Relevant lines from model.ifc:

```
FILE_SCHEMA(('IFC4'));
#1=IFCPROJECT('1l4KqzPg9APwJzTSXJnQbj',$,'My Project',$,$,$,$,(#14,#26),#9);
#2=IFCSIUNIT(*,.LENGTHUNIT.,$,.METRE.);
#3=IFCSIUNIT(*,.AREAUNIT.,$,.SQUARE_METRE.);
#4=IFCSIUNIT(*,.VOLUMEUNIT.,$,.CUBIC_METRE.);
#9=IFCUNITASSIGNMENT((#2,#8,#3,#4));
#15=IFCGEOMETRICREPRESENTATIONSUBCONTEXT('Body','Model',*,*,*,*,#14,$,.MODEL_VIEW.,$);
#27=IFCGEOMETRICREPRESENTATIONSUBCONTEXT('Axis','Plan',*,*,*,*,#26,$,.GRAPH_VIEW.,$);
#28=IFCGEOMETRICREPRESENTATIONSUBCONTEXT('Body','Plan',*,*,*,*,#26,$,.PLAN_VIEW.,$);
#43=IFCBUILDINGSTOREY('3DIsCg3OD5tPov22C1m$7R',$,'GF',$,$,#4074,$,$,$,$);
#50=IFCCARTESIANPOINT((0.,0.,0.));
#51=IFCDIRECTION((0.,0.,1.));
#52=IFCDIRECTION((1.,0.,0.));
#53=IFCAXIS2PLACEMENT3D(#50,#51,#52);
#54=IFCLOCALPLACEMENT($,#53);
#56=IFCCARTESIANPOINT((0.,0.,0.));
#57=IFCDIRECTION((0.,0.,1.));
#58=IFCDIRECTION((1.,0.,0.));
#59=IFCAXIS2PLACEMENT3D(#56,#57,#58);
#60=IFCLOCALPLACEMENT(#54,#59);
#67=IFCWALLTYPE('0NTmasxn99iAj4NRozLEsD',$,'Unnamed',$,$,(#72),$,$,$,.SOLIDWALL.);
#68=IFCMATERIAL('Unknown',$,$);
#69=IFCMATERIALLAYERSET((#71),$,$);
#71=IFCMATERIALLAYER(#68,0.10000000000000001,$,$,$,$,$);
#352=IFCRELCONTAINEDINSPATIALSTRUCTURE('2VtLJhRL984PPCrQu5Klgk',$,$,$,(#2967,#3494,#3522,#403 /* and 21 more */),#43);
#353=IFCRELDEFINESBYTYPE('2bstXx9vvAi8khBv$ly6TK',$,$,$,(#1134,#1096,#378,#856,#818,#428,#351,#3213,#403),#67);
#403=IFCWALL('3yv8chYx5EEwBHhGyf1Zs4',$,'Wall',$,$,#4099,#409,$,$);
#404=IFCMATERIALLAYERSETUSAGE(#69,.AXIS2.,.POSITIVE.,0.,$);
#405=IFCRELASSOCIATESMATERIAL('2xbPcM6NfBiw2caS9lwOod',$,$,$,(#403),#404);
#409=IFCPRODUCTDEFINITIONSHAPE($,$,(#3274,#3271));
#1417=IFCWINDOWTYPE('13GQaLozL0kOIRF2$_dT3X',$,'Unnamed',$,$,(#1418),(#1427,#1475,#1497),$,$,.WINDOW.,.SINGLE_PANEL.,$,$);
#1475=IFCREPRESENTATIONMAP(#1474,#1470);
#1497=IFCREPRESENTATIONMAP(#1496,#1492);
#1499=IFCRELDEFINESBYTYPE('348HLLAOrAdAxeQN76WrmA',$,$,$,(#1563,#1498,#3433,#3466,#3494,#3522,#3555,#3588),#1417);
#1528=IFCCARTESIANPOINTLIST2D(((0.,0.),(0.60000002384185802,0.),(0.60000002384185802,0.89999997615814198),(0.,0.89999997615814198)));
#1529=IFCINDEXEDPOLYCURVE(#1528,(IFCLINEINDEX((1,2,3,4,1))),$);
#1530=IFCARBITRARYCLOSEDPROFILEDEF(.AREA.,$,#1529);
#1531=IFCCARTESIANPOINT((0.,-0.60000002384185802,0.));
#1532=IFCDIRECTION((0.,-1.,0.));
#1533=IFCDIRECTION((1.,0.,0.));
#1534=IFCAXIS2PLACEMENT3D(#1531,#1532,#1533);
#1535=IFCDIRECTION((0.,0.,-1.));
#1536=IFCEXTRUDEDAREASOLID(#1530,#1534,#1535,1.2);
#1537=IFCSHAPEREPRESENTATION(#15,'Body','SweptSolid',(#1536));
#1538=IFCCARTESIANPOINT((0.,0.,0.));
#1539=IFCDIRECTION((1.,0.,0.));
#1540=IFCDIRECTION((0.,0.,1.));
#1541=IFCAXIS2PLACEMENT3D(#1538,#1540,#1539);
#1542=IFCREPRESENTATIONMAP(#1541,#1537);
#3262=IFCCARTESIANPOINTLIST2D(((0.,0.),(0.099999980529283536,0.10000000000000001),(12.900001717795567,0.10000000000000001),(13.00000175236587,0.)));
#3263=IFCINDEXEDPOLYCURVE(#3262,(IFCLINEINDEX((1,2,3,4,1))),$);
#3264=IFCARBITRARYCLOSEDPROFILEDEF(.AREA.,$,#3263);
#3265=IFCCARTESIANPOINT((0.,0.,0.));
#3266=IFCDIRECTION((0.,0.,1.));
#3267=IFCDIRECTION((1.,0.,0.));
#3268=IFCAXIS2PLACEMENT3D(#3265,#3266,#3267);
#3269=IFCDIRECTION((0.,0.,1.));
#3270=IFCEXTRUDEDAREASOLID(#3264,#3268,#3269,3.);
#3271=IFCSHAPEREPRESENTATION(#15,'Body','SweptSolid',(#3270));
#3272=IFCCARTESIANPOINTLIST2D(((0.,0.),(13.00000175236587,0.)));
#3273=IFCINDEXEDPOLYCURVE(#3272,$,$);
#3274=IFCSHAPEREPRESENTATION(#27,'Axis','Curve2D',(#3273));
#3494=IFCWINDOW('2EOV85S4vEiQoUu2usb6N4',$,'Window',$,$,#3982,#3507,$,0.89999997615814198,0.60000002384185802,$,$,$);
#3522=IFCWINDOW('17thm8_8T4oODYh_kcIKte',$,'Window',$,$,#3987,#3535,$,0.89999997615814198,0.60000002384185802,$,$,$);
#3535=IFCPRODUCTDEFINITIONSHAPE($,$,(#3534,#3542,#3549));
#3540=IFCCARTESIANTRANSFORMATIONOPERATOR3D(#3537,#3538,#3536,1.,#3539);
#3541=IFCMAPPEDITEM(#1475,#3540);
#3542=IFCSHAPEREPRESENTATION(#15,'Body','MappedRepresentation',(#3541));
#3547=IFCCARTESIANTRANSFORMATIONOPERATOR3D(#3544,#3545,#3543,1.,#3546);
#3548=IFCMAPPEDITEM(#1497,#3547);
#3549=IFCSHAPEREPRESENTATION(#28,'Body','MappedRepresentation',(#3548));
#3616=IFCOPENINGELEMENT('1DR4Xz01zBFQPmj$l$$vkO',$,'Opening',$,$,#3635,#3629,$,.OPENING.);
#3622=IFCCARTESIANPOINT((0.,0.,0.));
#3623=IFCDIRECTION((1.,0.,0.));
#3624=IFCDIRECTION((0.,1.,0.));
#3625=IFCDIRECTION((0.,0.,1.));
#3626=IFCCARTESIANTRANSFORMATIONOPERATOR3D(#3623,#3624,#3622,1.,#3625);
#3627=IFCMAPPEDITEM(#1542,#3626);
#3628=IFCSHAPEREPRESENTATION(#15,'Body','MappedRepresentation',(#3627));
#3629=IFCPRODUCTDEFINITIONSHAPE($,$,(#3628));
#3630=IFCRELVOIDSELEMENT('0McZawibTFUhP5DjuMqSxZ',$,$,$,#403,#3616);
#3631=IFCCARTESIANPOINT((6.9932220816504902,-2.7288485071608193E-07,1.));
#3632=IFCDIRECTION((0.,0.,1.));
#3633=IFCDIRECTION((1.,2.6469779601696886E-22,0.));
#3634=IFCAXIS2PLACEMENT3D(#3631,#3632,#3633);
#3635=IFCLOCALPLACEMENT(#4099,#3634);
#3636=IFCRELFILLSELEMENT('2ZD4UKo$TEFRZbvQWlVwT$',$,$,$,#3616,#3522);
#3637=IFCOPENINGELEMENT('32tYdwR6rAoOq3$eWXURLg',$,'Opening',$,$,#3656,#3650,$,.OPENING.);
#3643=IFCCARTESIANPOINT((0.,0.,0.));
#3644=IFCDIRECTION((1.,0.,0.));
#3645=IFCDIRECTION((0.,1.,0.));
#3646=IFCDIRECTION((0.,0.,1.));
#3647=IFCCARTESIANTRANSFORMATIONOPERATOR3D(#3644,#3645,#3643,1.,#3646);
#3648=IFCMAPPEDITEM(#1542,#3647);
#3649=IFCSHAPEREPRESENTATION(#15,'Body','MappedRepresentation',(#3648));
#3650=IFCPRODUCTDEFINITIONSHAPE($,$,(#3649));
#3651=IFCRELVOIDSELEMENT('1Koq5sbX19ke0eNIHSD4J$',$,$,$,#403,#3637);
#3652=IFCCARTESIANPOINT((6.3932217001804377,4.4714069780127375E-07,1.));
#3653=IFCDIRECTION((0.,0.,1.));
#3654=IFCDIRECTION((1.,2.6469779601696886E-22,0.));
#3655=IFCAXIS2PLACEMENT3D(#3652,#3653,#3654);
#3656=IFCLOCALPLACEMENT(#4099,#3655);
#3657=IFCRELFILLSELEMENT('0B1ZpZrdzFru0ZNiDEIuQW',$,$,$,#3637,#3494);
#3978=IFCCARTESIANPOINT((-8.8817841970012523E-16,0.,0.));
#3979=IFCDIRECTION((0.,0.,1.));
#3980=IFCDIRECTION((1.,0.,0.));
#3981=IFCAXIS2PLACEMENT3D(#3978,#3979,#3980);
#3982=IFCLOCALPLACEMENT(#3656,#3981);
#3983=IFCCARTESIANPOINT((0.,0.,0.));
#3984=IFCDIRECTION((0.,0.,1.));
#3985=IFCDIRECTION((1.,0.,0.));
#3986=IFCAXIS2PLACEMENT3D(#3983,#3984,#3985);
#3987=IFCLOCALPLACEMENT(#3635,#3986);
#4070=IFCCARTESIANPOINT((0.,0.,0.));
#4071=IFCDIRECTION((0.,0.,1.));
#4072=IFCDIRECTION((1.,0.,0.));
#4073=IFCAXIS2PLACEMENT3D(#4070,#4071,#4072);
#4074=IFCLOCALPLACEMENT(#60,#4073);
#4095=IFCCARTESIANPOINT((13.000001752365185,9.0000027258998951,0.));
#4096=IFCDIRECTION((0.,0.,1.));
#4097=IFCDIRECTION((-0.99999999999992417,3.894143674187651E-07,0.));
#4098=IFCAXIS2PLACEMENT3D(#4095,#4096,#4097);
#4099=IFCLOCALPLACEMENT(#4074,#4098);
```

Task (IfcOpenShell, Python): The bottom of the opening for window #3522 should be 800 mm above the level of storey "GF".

```python
import numpy as np
import ifcopenshell
import ifcopenshell.api.geometry
import ifcopenshell.geom
import ifcopenshell.util.element
import ifcopenshell.util.placement
import ifcopenshell.util.shape
import ifcopenshell.util.unit

model = ifcopenshell.open("model.ifc")
unit_scale = ifcopenshell.util.unit.calculate_unit_scale(model)

window = model.by_id(3522)
opening = window.FillsVoids[0].RelatingOpeningElement
storey = ifcopenshell.util.element.get_container(window, ifc_class="IfcBuildingStorey")
level = ifcopenshell.util.placement.get_local_placement(storey.ObjectPlacement)[2, 3]

# The opening's origin need not be at the sill, so measure its lowest point.
shape = ifcopenshell.geom.create_shape(ifcopenshell.geom.settings(), opening)
bottom = ifcopenshell.util.shape.get_shape_bottom_elevation(shape, shape.geometry) / unit_scale
dz = level + 0.8 / unit_scale - bottom

shift = np.array([0.0, 0.0, dz])
# The window is placed relative to its opening, so it follows when the opening moves.
matrix = ifcopenshell.util.placement.get_local_placement(opening.ObjectPlacement)
matrix[:3, 3] += shift
ifcopenshell.api.geometry.edit_object_placement(
    model, product=opening, matrix=matrix, is_si=False, should_transform_children=True
)

print(f"moved by {dz * unit_scale:+.3f} m")

model.write("model_rev.ifc")
```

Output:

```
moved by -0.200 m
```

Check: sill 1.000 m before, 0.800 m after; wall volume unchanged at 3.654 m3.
